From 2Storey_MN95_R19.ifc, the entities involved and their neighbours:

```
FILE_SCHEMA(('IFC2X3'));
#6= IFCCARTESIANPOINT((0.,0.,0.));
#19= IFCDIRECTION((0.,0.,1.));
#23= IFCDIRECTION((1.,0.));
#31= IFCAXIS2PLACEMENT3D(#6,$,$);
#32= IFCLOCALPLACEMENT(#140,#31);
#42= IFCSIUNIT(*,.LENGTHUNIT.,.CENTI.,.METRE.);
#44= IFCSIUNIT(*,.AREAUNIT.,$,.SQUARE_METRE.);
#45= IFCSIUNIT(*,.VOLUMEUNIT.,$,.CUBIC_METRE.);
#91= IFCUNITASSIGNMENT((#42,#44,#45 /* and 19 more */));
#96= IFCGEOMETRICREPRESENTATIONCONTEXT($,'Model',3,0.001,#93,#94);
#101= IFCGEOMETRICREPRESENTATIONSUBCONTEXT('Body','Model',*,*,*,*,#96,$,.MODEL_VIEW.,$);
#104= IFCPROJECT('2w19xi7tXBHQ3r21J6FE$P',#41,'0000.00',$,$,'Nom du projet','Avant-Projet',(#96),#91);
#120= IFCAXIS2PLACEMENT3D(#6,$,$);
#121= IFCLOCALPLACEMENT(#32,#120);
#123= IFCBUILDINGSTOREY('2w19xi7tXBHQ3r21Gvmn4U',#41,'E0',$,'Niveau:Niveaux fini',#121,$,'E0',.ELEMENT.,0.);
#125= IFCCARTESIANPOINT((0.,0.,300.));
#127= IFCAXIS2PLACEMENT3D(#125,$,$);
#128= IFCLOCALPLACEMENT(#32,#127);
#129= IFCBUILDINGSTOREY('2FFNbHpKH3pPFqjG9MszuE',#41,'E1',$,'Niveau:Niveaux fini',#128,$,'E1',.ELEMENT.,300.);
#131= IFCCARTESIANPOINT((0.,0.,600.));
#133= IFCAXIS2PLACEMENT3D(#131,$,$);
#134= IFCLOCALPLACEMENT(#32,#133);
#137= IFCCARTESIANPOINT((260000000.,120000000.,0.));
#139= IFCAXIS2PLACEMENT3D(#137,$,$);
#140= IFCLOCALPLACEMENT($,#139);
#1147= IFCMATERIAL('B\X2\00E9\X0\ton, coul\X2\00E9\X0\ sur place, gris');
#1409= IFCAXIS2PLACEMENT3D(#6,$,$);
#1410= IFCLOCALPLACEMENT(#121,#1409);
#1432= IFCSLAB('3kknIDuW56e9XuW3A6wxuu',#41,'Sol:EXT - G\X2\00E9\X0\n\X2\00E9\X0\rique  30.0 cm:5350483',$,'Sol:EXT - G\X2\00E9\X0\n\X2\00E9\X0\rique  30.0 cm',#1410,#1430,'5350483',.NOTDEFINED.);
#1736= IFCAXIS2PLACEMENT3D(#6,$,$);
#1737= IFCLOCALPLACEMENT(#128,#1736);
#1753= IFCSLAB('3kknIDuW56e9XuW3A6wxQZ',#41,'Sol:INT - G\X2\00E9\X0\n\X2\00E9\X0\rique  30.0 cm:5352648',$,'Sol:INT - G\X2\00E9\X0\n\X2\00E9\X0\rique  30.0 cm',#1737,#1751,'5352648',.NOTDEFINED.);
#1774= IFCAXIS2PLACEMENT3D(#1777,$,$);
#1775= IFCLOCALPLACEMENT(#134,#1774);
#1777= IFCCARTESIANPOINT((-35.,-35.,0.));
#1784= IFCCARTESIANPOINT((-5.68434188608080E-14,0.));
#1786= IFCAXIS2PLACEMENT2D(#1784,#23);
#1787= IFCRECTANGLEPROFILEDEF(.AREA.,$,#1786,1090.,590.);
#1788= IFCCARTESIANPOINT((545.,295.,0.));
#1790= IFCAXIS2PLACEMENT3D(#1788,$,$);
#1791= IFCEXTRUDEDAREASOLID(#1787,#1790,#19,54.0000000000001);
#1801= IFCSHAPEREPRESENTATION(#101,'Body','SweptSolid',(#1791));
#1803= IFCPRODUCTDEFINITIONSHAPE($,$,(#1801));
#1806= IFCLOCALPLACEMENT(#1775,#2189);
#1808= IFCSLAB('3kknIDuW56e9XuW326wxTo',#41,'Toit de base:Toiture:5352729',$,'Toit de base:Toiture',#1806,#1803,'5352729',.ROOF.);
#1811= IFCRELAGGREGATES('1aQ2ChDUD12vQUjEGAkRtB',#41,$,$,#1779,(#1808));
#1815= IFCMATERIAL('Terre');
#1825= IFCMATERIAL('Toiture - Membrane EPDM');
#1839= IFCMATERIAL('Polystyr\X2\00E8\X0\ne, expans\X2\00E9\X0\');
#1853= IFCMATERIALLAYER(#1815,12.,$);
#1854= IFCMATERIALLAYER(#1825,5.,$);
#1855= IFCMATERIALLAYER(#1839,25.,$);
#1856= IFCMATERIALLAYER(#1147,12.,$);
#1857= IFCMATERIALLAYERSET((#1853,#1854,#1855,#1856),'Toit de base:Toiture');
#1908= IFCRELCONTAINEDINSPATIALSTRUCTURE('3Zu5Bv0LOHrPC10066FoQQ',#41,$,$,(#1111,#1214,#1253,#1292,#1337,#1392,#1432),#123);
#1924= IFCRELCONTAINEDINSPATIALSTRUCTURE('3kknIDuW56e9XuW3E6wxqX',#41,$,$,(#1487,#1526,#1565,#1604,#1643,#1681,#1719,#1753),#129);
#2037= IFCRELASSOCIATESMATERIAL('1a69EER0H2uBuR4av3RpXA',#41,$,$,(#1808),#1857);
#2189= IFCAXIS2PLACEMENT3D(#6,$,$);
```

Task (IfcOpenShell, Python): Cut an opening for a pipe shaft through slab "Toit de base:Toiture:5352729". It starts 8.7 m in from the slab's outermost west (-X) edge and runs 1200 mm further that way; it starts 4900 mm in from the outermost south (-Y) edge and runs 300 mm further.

```python
import numpy as np
import ifcopenshell
import ifcopenshell.api.feature
import ifcopenshell.api.geometry
import ifcopenshell.api.root
import ifcopenshell.geom
import ifcopenshell.util.placement
import ifcopenshell.util.representation
import ifcopenshell.util.shape
import ifcopenshell.util.unit

model = ifcopenshell.open("2Storey_MN95_R19.ifc")
unit_scale = ifcopenshell.util.unit.calculate_unit_scale(model)
settings = ifcopenshell.geom.settings()


def volume(element):
    """Net volume in cubic metres, openings subtracted."""
    shape = ifcopenshell.geom.create_shape(settings, element)
    return ifcopenshell.util.shape.get_volume(shape.geometry)


slab = model.by_id(1808)
before = volume(slab)

# Extent in the slab's own axes, in metres. The edges named are its -X and -Y sides.
slab_shape = ifcopenshell.geom.create_shape(settings, slab)
vertices = ifcopenshell.util.shape.get_vertices(slab_shape.geometry)
x_min, y_min, bottom = vertices.min(axis=0)
top = vertices[:, 2].max()

opening = ifcopenshell.api.root.create_entity(model, ifc_class="IfcOpeningElement", name="Pipe shaft opening")
context = ifcopenshell.util.representation.get_context(model, "Model", "Body", "MODEL_VIEW")
width, depth = 1.2, 0.3
outline = [(0.0, 0.0), (width, 0.0), (width, depth), (0.0, depth), (0.0, 0.0)]
# Overshoot both faces by 50 mm so the cut is clean.
shape = ifcopenshell.api.geometry.add_slab_representation(
    model, context=context, depth=top - bottom + 0.1, polyline=outline
)
ifcopenshell.api.geometry.assign_representation(model, product=opening, representation=shape)

matrix = ifcopenshell.util.placement.get_local_placement(slab.ObjectPlacement)
matrix[:, 3] = matrix @ np.append(np.array([x_min + 8.7, y_min + 4.9, bottom - 0.05]) / unit_scale, 1.0)
ifcopenshell.api.geometry.edit_object_placement(model, product=opening, matrix=matrix, is_si=False)
ifcopenshell.api.feature.add_feature(model, feature=opening, element=slab)

after = volume(slab)

print(f"slab volume {before:.3f} -> {after:.3f} m3")

model.write("2Storey_MN95_R19-out.ifc")
```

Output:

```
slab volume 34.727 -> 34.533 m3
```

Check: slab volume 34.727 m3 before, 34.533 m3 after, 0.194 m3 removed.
